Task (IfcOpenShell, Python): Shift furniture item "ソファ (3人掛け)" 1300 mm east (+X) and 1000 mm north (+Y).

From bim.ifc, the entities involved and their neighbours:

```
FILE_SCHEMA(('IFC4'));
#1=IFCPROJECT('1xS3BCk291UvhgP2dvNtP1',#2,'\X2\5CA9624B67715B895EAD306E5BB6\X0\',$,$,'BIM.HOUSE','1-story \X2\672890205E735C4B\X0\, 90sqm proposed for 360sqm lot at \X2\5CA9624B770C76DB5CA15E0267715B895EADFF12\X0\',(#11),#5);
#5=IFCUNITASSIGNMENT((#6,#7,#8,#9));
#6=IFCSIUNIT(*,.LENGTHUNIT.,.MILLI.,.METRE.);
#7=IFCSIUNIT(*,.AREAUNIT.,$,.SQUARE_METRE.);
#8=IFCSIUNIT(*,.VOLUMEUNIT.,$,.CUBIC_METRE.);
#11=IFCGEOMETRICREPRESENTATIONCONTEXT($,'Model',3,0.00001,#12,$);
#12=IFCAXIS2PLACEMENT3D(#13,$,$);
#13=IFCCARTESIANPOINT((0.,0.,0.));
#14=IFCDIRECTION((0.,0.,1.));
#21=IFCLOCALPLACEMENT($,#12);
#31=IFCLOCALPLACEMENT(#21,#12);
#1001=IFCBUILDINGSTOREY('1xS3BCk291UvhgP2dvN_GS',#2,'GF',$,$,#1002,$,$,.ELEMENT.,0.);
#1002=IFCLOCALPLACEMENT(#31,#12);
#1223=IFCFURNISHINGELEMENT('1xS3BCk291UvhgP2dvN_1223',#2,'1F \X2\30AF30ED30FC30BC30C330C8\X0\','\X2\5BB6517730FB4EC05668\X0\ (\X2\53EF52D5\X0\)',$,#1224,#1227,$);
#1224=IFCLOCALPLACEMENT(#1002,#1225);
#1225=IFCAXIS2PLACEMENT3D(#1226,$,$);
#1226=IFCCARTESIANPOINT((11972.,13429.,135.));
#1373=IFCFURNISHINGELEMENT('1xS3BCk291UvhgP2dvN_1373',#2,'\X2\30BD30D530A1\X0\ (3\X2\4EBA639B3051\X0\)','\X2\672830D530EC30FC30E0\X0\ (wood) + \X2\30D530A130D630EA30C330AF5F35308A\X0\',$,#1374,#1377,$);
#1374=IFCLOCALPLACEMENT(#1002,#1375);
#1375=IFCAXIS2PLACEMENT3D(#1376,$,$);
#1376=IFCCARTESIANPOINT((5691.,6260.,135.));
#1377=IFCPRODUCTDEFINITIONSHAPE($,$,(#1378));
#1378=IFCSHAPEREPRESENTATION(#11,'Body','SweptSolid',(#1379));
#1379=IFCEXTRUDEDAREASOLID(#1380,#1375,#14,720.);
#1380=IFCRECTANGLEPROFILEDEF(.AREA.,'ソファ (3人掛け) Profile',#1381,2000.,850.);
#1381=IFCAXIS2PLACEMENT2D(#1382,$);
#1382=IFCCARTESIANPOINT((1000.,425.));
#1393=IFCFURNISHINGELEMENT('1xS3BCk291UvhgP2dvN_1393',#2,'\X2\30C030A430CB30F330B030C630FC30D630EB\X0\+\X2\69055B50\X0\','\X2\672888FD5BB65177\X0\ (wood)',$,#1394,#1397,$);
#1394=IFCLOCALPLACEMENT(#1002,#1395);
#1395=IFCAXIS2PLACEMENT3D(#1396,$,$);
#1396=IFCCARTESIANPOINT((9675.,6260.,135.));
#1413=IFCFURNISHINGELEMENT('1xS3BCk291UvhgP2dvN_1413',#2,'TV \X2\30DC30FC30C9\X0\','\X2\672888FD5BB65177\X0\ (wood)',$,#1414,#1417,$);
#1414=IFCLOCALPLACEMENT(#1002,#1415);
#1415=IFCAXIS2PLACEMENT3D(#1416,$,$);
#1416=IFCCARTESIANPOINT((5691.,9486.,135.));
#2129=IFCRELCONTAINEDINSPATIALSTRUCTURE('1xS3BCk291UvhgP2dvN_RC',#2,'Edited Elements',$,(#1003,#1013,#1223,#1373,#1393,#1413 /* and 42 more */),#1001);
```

```python
import ifcopenshell
import ifcopenshell.api.geometry
import ifcopenshell.util.placement
import ifcopenshell.util.unit

model = ifcopenshell.open("bim.ifc")
unit_scale = ifcopenshell.util.unit.calculate_unit_scale(model)

item = model.by_guid("1xS3BCk291UvhgP2dvN_1373")
matrix = ifcopenshell.util.placement.get_local_placement(item.ObjectPlacement)
matrix[0, 3] += 1.3 / unit_scale
matrix[1, 3] += 1 / unit_scale
ifcopenshell.api.geometry.edit_object_placement(model, product=item, matrix=matrix, is_si=False)

print(ifcopenshell.util.placement.get_local_placement(item.ObjectPlacement).round(3) + 0.0)

model.write("bim_updated.ifc")
```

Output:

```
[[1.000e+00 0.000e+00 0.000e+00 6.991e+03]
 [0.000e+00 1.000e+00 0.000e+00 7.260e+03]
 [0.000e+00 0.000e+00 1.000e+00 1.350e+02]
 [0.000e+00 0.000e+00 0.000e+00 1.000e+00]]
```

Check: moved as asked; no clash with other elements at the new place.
